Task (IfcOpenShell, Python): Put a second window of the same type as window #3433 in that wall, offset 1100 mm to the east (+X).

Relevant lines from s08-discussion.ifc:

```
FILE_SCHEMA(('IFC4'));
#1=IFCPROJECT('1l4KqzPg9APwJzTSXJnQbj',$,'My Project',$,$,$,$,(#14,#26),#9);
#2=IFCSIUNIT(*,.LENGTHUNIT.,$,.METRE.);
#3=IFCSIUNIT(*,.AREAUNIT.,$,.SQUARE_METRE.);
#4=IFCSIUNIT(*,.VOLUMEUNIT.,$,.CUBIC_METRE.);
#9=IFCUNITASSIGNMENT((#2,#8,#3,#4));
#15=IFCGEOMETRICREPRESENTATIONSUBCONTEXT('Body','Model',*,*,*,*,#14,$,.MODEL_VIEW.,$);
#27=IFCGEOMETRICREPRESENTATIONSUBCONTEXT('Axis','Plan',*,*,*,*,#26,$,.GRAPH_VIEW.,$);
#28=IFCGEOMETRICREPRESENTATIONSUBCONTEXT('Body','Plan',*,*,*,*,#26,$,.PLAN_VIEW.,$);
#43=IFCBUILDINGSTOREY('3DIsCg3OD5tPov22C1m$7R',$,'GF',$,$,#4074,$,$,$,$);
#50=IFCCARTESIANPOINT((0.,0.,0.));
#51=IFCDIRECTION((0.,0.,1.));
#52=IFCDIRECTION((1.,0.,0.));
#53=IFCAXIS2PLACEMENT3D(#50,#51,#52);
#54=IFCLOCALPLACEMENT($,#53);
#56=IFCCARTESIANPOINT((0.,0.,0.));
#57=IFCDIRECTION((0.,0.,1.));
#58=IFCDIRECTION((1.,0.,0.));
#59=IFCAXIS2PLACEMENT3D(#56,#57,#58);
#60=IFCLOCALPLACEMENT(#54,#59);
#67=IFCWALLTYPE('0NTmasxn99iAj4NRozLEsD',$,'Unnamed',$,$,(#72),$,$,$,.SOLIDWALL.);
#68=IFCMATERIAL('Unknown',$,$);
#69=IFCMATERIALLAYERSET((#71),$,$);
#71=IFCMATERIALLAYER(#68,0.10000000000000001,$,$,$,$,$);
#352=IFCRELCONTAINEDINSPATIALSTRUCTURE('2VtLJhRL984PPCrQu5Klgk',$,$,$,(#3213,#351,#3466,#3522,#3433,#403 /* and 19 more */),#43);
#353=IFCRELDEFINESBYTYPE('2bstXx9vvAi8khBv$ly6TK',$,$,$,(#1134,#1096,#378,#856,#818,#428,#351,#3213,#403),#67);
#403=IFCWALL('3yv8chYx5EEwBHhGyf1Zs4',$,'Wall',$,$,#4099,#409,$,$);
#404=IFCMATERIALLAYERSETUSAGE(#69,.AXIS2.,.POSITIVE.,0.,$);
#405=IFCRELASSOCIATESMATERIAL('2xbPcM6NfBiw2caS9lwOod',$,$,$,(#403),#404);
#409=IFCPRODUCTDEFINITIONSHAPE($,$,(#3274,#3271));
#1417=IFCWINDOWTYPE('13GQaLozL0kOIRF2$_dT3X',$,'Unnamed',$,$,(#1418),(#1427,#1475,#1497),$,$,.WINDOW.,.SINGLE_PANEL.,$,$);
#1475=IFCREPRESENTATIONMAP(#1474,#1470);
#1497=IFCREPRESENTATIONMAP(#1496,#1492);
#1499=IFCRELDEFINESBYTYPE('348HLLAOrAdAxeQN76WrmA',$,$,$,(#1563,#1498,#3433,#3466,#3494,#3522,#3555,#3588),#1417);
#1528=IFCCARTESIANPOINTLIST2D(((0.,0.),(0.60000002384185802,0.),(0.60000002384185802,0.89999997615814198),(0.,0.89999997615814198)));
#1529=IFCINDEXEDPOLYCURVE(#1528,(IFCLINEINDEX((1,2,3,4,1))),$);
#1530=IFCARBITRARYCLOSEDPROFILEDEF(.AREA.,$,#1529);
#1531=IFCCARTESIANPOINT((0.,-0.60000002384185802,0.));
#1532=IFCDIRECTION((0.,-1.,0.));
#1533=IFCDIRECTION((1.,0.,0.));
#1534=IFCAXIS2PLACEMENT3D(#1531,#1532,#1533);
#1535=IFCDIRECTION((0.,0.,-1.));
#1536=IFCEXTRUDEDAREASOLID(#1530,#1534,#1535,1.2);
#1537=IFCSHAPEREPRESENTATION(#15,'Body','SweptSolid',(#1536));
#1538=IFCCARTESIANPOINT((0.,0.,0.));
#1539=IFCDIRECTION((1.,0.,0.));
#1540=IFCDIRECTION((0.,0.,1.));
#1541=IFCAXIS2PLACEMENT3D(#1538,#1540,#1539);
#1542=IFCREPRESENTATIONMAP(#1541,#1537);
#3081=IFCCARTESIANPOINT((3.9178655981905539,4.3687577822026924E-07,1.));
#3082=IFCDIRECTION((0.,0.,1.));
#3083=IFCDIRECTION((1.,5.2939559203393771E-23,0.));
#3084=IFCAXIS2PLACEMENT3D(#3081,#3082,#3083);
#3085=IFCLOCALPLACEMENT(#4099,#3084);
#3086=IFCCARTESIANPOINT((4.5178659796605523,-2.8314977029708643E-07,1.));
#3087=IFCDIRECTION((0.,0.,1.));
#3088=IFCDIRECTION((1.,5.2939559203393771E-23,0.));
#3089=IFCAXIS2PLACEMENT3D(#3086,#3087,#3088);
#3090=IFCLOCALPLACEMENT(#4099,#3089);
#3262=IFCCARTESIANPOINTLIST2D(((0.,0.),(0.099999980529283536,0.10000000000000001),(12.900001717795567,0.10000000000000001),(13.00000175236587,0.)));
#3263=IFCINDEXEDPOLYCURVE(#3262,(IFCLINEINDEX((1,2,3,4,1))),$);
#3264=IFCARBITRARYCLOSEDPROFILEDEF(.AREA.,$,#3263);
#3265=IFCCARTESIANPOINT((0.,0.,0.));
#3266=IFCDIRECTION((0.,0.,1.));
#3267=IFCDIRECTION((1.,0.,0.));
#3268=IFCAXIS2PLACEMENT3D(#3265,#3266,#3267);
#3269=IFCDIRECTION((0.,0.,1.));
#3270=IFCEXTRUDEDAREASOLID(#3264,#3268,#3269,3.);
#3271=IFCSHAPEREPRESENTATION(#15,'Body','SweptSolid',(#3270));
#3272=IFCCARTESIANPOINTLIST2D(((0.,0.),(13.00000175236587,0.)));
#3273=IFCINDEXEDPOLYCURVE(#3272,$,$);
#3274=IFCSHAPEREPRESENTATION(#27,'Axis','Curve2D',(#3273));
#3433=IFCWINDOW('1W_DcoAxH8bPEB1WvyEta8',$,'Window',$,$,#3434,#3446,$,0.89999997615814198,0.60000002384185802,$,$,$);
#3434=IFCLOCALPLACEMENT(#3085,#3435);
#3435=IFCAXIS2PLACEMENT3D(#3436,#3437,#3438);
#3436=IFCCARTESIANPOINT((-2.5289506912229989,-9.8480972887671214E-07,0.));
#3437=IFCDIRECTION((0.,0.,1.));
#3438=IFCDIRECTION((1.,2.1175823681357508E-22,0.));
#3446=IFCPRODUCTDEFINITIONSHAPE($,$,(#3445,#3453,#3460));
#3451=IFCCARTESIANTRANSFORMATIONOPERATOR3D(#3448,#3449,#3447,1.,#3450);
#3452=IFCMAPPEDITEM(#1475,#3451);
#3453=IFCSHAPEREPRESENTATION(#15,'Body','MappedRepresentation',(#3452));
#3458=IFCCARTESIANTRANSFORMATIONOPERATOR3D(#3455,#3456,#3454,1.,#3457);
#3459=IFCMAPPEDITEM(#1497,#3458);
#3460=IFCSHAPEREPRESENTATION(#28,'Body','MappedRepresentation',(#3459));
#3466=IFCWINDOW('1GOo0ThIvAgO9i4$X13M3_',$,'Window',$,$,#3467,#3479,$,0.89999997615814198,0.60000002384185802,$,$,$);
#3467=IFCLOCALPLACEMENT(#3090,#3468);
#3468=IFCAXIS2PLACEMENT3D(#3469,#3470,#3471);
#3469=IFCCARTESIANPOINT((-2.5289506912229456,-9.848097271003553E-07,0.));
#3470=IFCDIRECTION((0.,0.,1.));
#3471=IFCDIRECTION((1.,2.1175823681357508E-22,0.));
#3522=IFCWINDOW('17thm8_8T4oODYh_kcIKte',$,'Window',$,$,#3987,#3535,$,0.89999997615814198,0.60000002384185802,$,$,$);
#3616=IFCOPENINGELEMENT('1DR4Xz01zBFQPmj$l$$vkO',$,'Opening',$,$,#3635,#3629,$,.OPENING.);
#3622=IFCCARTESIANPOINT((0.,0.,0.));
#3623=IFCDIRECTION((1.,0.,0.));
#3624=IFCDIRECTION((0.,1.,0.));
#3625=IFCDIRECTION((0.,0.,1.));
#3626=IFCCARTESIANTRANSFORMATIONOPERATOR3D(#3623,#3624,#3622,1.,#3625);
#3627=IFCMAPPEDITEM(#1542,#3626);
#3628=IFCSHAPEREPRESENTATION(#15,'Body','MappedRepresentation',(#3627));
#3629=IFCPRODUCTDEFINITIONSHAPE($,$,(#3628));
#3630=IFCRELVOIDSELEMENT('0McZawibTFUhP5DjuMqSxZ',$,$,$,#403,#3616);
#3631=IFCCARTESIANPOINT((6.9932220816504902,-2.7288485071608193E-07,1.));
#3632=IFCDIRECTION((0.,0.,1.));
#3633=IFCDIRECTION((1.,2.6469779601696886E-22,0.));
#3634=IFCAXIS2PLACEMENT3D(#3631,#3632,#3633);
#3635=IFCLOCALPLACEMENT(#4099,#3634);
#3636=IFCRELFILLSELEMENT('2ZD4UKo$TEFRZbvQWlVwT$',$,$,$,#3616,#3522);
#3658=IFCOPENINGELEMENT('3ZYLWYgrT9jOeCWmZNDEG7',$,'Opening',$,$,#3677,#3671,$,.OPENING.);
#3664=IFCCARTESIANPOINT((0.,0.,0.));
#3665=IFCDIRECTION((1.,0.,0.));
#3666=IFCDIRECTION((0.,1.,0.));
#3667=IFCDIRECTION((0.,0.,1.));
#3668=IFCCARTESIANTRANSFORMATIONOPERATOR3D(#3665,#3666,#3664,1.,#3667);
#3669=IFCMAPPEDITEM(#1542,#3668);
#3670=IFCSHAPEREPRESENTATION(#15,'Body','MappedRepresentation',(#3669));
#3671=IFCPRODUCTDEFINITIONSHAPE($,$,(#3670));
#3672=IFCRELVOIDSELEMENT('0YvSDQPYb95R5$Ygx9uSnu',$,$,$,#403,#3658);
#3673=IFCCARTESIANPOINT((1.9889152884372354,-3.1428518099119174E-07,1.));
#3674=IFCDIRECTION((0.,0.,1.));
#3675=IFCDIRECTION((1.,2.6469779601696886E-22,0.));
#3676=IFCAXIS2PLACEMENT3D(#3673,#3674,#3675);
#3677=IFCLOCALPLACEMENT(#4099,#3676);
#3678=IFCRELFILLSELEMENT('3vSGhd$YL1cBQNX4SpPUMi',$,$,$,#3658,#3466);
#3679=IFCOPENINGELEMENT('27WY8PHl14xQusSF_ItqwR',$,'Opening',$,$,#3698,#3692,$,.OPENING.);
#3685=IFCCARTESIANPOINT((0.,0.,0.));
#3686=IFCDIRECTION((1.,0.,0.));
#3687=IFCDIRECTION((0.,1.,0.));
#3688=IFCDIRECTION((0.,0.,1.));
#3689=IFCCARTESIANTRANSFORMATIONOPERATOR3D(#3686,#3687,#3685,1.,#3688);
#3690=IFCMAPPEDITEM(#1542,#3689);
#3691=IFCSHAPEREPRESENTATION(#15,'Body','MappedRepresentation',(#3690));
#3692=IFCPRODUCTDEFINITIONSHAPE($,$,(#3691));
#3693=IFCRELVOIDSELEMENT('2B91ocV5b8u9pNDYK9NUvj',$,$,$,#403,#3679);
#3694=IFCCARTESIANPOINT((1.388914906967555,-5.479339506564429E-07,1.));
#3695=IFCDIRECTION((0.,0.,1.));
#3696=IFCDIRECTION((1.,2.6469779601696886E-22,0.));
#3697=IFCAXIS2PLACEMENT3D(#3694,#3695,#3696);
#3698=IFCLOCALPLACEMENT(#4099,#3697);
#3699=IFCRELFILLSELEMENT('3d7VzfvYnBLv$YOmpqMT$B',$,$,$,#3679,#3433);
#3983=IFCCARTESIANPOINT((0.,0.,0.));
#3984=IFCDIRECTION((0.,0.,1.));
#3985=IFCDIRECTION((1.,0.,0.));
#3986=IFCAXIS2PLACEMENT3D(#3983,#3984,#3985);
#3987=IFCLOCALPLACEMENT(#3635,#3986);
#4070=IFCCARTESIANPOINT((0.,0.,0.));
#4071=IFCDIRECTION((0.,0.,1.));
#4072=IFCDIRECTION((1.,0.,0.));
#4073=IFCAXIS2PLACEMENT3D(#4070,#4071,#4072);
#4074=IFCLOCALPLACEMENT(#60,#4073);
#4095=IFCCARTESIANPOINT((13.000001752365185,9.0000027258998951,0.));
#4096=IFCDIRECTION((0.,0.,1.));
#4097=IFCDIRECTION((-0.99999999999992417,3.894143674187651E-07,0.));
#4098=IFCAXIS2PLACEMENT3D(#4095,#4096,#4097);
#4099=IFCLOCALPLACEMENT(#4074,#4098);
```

```python
import ifcopenshell
import ifcopenshell.api.feature
import ifcopenshell.api.geometry
import ifcopenshell.api.root
import ifcopenshell.geom
import ifcopenshell.util.element
import ifcopenshell.util.placement
import ifcopenshell.util.shape
import ifcopenshell.util.unit

model = ifcopenshell.open("s08-discussion.ifc")
unit_scale = ifcopenshell.util.unit.calculate_unit_scale(model)
settings = ifcopenshell.geom.settings()


def volume(element):
    """Net volume in cubic metres, openings subtracted."""
    shape = ifcopenshell.geom.create_shape(settings, element)
    return ifcopenshell.util.shape.get_volume(shape.geometry)


window = model.by_id(3433)
opening = window.FillsVoids[0].RelatingOpeningElement
wall = opening.VoidsElements[0].RelatingBuildingElement
before = volume(wall)
shift = ifcopenshell.util.placement.get_local_placement(wall.ObjectPlacement)[:3, 0] * -1.1 / unit_scale

# copy_class copies the void relationship, type, container and properties, but no geometry.
new_opening = ifcopenshell.api.root.copy_class(model, product=opening)
new_opening.Representation = ifcopenshell.util.element.copy_deep(
    model, opening.Representation, exclude=["IfcGeometricRepresentationContext", "IfcRepresentationMap"]
)
new_window = ifcopenshell.api.root.copy_class(model, product=window)
new_window.Representation = ifcopenshell.util.element.copy_deep(
    model, window.Representation, exclude=["IfcGeometricRepresentationContext", "IfcRepresentationMap"]
)
ifcopenshell.api.feature.add_filling(model, opening=new_opening, element=new_window)

for old, new in ((opening, new_opening), (window, new_window)):
    matrix = ifcopenshell.util.placement.get_local_placement(old.ObjectPlacement)
    matrix[:3, 3] += shift
    ifcopenshell.api.geometry.edit_object_placement(model, product=new, matrix=matrix, is_si=False)

after = volume(wall)

print(f"wall volume {before:.3f} -> {after:.3f} m3")

model.write("s08-discussion_edited.ifc")
```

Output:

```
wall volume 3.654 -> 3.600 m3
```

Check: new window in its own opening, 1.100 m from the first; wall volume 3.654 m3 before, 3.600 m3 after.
